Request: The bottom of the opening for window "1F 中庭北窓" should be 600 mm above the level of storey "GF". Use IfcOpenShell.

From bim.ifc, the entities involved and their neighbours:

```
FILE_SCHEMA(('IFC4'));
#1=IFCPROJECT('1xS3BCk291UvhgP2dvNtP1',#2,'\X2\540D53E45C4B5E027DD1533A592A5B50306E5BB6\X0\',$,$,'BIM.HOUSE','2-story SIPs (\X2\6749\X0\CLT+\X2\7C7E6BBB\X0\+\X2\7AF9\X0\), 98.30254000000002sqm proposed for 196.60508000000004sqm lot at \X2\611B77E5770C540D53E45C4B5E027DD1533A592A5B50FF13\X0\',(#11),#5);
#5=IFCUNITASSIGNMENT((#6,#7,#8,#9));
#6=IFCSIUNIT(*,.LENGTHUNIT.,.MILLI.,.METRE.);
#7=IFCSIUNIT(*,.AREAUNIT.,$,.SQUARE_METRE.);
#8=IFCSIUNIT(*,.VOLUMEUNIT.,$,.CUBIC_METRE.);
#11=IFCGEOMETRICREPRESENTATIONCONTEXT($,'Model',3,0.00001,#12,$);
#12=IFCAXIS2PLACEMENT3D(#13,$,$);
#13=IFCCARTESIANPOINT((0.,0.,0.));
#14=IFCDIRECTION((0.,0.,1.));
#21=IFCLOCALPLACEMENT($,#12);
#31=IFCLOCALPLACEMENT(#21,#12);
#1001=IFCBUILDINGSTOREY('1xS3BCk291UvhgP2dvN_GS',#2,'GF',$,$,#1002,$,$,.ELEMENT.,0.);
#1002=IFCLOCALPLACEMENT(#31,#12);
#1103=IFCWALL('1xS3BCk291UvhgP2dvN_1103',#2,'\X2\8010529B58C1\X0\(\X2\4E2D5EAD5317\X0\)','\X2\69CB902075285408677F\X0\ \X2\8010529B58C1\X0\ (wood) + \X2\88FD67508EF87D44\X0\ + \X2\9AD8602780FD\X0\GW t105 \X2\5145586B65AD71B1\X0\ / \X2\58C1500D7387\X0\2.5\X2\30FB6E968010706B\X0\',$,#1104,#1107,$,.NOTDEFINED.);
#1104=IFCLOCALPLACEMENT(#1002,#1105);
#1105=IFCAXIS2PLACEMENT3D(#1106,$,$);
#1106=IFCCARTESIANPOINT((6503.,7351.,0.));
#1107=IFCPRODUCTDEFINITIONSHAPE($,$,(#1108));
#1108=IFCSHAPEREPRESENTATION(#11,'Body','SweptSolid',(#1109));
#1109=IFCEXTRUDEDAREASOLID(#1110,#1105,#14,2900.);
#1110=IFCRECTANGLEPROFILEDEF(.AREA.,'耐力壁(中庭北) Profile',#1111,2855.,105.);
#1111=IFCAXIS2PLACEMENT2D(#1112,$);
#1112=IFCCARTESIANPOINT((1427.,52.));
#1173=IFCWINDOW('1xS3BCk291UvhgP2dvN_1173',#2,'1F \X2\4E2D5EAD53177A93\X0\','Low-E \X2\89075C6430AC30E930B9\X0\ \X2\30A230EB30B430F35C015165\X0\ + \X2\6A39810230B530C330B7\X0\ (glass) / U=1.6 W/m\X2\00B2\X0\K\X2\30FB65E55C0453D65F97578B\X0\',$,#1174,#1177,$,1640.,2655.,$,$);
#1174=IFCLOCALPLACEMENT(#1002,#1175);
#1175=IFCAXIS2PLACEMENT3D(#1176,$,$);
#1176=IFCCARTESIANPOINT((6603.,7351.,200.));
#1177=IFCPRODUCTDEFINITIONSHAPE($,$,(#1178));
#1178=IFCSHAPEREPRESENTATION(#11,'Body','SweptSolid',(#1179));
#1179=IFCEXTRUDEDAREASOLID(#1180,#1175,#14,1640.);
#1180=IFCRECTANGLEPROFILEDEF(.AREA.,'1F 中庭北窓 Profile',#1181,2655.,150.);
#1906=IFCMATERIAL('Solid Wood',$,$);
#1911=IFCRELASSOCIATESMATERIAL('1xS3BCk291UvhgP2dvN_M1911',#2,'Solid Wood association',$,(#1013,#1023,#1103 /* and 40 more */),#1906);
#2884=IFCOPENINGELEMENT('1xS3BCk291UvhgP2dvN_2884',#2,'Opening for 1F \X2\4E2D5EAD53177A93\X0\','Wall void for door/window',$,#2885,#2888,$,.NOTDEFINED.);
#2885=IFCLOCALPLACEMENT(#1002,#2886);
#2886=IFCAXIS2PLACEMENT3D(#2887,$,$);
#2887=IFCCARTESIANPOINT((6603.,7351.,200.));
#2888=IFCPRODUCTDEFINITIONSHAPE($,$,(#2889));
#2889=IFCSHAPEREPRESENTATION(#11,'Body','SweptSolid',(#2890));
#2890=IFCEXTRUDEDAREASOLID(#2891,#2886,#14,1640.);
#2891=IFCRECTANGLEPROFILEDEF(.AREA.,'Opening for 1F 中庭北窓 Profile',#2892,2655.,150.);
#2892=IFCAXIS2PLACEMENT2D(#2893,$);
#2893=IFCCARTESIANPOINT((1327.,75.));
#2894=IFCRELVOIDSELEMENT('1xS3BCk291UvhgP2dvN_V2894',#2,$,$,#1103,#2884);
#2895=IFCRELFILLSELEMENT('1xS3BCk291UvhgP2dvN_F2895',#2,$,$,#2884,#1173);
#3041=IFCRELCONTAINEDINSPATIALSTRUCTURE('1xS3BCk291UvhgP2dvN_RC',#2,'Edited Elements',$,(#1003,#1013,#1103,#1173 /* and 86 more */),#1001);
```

```python
import numpy as np
import ifcopenshell
import ifcopenshell.api.geometry
import ifcopenshell.geom
import ifcopenshell.util.element
import ifcopenshell.util.placement
import ifcopenshell.util.shape
import ifcopenshell.util.unit

model = ifcopenshell.open("bim.ifc")
unit_scale = ifcopenshell.util.unit.calculate_unit_scale(model)

window = model.by_guid("1xS3BCk291UvhgP2dvN_1173")
opening = window.FillsVoids[0].RelatingOpeningElement
storey = ifcopenshell.util.element.get_container(window, ifc_class="IfcBuildingStorey")
level = ifcopenshell.util.placement.get_local_placement(storey.ObjectPlacement)[2, 3]

# The opening's origin need not be at the sill, so measure its lowest point.
shape = ifcopenshell.geom.create_shape(ifcopenshell.geom.settings(), opening)
bottom = ifcopenshell.util.shape.get_shape_bottom_elevation(shape, shape.geometry) / unit_scale
dz = level + 0.6 / unit_scale - bottom

shift = np.array([0.0, 0.0, dz])
# The window is not placed relative to its opening, so move both.
for product in (opening, window):
    matrix = ifcopenshell.util.placement.get_local_placement(product.ObjectPlacement)
    matrix[:3, 3] += shift
    ifcopenshell.api.geometry.edit_object_placement(model, product=product, matrix=matrix, is_si=False)

print(f"moved by {dz * unit_scale:+.3f} m")

model.write("bim-out.ifc")
```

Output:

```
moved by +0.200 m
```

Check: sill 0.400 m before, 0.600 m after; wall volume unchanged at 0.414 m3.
